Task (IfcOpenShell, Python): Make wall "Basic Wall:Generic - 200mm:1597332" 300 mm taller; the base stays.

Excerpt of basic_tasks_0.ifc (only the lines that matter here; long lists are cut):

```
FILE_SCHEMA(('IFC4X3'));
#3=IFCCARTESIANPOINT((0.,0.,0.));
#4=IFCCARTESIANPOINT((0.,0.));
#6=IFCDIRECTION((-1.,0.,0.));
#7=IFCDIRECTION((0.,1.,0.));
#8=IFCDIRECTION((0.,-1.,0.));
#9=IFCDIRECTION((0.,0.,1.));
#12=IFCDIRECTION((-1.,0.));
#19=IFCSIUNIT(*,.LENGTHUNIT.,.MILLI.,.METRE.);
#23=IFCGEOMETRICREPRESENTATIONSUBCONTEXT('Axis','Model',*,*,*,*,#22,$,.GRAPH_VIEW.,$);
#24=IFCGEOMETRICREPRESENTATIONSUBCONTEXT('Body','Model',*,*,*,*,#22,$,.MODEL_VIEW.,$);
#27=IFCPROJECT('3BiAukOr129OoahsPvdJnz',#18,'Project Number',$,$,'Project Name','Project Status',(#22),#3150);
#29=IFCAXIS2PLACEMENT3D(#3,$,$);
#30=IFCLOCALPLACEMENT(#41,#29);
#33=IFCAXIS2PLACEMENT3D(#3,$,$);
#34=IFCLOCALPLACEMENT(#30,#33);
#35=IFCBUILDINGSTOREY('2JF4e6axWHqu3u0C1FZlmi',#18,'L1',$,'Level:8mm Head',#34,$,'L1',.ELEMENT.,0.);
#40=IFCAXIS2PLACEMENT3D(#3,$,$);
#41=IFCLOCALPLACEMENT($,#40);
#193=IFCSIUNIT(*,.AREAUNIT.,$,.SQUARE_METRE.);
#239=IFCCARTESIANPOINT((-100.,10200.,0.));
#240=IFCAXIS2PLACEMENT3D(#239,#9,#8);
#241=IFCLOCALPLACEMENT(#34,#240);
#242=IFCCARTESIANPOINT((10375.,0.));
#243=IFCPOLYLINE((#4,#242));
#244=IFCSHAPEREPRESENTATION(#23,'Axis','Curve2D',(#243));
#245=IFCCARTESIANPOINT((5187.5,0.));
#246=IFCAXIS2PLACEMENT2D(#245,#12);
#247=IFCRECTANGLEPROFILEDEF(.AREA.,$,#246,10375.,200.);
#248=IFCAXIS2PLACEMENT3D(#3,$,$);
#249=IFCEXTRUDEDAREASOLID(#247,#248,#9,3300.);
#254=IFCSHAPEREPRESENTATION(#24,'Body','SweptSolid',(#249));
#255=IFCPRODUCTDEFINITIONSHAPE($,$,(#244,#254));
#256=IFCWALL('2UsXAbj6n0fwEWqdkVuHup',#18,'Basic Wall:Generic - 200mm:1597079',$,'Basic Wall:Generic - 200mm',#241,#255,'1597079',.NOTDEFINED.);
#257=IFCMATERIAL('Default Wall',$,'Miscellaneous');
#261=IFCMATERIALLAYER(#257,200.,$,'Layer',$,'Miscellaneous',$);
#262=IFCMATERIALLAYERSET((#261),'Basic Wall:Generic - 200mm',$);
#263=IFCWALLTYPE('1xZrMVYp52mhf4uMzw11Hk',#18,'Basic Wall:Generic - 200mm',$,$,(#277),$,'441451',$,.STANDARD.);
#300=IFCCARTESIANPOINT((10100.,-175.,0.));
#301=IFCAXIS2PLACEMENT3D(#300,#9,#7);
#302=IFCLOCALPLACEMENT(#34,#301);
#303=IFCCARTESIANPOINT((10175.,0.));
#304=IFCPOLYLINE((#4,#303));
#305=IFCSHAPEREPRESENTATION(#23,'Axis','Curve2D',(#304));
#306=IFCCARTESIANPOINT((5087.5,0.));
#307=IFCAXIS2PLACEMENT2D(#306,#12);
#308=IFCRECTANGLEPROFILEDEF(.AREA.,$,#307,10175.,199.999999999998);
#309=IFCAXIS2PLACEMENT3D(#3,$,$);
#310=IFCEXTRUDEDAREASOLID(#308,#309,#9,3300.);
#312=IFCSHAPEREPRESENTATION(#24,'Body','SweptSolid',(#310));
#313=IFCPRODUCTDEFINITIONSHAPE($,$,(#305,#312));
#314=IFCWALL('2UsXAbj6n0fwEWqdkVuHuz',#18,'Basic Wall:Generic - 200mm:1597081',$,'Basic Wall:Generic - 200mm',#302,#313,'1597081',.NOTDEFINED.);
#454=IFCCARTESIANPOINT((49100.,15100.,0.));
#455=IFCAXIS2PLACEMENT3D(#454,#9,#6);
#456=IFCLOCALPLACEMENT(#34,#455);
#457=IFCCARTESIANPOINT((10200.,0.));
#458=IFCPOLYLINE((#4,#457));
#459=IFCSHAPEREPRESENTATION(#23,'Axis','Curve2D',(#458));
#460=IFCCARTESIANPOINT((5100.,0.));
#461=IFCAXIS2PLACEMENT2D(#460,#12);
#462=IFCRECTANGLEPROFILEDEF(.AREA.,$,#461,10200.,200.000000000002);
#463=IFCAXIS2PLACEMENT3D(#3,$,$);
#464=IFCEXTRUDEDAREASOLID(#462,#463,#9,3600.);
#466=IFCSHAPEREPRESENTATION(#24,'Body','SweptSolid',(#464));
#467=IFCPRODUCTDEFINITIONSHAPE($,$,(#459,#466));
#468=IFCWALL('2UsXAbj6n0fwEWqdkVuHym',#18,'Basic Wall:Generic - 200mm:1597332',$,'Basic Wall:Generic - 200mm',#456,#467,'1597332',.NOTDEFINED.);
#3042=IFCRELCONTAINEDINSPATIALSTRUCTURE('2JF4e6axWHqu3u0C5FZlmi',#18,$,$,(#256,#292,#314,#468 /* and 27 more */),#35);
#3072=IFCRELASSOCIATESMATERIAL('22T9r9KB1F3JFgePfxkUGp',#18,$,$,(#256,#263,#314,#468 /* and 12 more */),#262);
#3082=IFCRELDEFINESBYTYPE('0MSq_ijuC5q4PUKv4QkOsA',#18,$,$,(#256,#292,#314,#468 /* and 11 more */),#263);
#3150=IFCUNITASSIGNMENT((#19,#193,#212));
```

```python
import ifcopenshell
import ifcopenshell.geom
import ifcopenshell.util.representation
import ifcopenshell.util.shape
import ifcopenshell.util.unit

model = ifcopenshell.open("basic_tasks_0.ifc")
unit_scale = ifcopenshell.util.unit.calculate_unit_scale(model)
settings = ifcopenshell.geom.settings()


def volume(element):
    """Net volume in cubic metres, openings subtracted."""
    shape = ifcopenshell.geom.create_shape(settings, element)
    return ifcopenshell.util.shape.get_volume(shape.geometry)


wall = model.by_guid("2UsXAbj6n0fwEWqdkVuHym")
before = volume(wall)

body = ifcopenshell.util.representation.get_representation(wall, "Model", "Body")
solid = body.Items[0]
old_height = solid.Depth
solid.Depth += 0.3 / unit_scale
after = volume(wall)

print(f"height {old_height:g} -> {solid.Depth:g}, volume {before:.3f} -> {after:.3f} m3")

model.write("basic_tasks_0_v2.ifc")
```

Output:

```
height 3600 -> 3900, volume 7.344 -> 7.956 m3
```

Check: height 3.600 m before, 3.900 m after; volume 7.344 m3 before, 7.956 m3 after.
